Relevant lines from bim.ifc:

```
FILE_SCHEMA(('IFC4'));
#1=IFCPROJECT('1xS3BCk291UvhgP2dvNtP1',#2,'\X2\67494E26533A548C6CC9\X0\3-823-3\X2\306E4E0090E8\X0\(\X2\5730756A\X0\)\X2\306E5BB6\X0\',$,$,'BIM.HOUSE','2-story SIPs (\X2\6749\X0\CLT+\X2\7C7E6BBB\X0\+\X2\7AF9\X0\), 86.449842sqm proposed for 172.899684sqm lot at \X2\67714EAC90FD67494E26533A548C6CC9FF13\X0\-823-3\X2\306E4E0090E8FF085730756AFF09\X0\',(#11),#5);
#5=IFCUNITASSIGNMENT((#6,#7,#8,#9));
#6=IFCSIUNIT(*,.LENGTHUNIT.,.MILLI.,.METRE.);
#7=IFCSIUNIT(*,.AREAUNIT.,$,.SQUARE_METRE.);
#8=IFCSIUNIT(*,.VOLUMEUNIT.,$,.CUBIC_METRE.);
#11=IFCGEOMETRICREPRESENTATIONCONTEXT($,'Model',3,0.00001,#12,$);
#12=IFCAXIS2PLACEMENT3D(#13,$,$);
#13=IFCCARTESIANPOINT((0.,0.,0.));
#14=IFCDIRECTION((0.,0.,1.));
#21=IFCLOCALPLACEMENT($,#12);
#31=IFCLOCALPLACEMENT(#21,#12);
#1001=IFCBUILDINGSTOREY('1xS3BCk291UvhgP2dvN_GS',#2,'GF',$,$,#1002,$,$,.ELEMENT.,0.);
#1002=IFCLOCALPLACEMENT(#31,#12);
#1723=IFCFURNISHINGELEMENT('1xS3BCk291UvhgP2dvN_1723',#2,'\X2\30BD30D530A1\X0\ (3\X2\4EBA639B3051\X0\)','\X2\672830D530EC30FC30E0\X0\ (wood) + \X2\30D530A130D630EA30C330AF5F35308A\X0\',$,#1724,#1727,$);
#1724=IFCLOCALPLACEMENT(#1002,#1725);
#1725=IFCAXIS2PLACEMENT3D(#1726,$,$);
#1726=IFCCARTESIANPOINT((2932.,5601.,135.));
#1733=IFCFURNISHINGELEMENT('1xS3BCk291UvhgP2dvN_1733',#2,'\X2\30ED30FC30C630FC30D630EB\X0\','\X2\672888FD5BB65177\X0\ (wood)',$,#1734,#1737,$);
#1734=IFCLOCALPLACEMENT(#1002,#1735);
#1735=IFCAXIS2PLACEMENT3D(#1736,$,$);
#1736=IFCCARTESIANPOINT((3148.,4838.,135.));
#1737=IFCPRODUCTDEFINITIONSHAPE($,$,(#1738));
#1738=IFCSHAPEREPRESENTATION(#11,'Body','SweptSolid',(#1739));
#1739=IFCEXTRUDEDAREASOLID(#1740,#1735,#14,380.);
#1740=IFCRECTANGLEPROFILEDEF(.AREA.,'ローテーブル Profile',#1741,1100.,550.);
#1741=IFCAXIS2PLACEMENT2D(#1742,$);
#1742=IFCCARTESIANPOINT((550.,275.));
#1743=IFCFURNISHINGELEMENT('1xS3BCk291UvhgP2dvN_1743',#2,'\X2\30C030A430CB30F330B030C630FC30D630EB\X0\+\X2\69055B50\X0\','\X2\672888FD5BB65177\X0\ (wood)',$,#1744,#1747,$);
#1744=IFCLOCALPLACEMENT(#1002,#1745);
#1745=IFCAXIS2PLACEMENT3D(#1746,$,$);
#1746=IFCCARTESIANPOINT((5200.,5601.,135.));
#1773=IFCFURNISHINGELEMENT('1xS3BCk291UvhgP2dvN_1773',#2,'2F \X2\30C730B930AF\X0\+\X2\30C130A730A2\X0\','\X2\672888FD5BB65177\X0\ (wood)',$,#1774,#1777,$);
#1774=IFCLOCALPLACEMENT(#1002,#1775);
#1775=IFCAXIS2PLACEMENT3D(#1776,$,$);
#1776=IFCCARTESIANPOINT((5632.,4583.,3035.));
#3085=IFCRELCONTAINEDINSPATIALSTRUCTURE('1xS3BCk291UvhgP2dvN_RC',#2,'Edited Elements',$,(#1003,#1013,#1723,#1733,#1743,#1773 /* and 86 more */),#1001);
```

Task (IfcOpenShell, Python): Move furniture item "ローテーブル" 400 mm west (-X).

```python
import ifcopenshell
import ifcopenshell.api.geometry
import ifcopenshell.util.placement
import ifcopenshell.util.unit

model = ifcopenshell.open("bim.ifc")
unit_scale = ifcopenshell.util.unit.calculate_unit_scale(model)

item = model.by_guid("1xS3BCk291UvhgP2dvN_1733")
matrix = ifcopenshell.util.placement.get_local_placement(item.ObjectPlacement)
matrix[0, 3] -= 0.4 / unit_scale
ifcopenshell.api.geometry.edit_object_placement(model, product=item, matrix=matrix, is_si=False)

print(ifcopenshell.util.placement.get_local_placement(item.ObjectPlacement).round(3) + 0.0)

model.write("bim_edited.ifc")
```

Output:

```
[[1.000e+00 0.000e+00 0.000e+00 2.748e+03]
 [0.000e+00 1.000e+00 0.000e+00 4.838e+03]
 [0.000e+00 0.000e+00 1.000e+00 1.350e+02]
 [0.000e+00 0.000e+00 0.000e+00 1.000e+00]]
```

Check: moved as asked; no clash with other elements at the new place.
